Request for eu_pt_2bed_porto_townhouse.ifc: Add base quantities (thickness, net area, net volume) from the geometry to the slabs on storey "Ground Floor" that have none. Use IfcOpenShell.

First a look at what the model holds.

```python
import ifcopenshell
import ifcopenshell.util.element
import ifcopenshell.util.unit

model = ifcopenshell.open("eu_pt_2bed_porto_townhouse.ifc")
print(model.schema)
for unit_type in ("LENGTHUNIT", "AREAUNIT", "VOLUMEUNIT"):
    print(unit_type, ifcopenshell.util.unit.calculate_unit_scale(model, unit_type))
storey = next(s for s in model.by_type("IfcBuildingStorey") if s.Name == "Ground Floor")
slabs = [e for e in ifcopenshell.util.element.get_decomposition(storey) if e.is_a("IfcSlab")]
for e in sorted(slabs, key=lambda e: e.id()):
    print(e.id(), e.is_a(), e.Name, list(ifcopenshell.util.element.get_psets(e, qtos_only=True)), sep=" | ")
```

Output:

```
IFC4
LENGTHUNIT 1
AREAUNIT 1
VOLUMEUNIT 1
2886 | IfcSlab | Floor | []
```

```python
import ifcopenshell
import ifcopenshell.api.pset
import ifcopenshell.geom
import ifcopenshell.util.element
import ifcopenshell.util.shape
import ifcopenshell.util.unit

model = ifcopenshell.open("eu_pt_2bed_porto_townhouse.ifc")
unit_scale = ifcopenshell.util.unit.calculate_unit_scale(model)
area_scale = ifcopenshell.util.unit.calculate_unit_scale(model, "AREAUNIT")
volume_scale = ifcopenshell.util.unit.calculate_unit_scale(model, "VOLUMEUNIT")
settings = ifcopenshell.geom.settings()

storey = next(s for s in model.by_type("IfcBuildingStorey") if s.Name == "Ground Floor")
slabs = [e for e in ifcopenshell.util.element.get_decomposition(storey) if e.is_a("IfcSlab")]

for e in sorted(slabs, key=lambda e: e.id()):
    if ifcopenshell.util.element.get_psets(e, qtos_only=True, should_inherit=False):
        continue
    # Geometry comes back in metres, in the element's own axes.
    shape = ifcopenshell.geom.create_shape(settings, e)
    values = {
        "Width": ifcopenshell.util.shape.get_z(shape.geometry) / unit_scale,
        "NetArea": ifcopenshell.util.shape.get_footprint_area(shape.geometry) / area_scale,
        "NetVolume": ifcopenshell.util.shape.get_volume(shape.geometry) / volume_scale,
    }
    qto = ifcopenshell.api.pset.add_qto(model, product=e, name="Qto_SlabBaseQuantities")
    ifcopenshell.api.pset.edit_qto(model, qto=qto, properties=values)
    print(e.id(), {k: round(v, 3) for k, v in values.items()})

model.write("eu_pt_2bed_porto_townhouse_v2.ifc")
```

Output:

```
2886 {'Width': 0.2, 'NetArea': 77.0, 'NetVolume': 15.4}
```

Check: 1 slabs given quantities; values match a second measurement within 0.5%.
